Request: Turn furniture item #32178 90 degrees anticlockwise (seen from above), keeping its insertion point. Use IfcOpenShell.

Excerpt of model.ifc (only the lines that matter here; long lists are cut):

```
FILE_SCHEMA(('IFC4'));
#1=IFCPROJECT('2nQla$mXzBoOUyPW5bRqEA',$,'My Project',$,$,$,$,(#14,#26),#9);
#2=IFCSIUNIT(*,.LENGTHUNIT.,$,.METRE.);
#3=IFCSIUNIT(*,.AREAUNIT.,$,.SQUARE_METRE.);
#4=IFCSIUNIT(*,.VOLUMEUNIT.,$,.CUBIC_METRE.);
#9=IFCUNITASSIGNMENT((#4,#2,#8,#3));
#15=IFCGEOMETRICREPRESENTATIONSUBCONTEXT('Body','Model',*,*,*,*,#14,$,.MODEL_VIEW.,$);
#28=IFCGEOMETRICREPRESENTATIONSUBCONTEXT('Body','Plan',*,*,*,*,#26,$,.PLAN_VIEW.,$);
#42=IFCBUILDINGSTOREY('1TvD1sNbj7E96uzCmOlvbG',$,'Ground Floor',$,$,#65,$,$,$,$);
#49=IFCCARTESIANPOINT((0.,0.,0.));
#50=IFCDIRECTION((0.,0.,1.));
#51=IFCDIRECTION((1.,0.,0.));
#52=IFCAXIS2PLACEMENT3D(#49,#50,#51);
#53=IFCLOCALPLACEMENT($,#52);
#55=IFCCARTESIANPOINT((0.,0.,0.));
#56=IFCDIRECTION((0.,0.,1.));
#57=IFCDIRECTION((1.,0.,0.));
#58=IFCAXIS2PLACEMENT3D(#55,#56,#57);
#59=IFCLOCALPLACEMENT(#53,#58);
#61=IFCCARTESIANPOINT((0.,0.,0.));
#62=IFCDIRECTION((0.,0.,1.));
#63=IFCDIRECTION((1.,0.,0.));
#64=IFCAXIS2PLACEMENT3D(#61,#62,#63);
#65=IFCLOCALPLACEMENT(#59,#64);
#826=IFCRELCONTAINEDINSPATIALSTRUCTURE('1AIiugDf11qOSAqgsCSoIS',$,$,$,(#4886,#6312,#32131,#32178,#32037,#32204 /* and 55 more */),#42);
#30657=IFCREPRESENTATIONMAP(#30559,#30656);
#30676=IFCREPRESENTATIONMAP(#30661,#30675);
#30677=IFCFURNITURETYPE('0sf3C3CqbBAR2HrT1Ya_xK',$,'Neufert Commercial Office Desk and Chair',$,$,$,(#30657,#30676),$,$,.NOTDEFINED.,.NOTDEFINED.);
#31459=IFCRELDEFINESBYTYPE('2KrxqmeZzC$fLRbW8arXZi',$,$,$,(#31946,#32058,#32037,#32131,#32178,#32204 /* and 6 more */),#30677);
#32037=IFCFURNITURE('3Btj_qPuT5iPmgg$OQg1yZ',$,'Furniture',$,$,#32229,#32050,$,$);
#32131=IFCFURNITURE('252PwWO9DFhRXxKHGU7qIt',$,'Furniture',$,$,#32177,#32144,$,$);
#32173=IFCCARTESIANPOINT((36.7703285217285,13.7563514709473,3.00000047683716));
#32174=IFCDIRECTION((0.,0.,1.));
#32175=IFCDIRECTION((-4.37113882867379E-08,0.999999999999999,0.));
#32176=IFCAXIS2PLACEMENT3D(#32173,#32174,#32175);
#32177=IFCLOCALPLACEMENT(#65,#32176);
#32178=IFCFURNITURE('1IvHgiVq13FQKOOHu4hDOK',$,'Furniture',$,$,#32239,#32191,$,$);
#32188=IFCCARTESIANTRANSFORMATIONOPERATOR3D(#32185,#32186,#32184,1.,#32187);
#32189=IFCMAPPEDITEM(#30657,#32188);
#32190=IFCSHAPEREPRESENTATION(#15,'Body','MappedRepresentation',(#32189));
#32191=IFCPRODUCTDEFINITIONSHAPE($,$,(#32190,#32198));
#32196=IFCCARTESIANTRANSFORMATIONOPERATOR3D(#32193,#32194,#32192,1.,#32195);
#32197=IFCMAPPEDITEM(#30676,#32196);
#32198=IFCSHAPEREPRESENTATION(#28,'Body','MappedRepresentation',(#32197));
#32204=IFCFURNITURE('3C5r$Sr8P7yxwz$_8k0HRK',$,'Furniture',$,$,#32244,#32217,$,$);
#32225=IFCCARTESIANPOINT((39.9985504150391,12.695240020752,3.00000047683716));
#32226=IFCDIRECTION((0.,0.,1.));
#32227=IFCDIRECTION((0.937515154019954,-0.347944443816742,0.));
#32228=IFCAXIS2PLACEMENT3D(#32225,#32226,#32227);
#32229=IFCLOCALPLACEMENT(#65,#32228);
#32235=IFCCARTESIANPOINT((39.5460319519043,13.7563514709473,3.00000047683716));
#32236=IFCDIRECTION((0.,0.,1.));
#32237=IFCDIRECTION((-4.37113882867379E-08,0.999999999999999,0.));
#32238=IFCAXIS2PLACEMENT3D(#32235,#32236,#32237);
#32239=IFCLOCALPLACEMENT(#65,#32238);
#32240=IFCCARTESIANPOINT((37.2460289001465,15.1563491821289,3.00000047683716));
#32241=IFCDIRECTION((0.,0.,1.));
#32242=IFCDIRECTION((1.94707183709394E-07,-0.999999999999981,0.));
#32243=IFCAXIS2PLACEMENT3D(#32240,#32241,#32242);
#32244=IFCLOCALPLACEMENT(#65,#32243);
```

```python
import ifcopenshell
import ifcopenshell.api.geometry
import ifcopenshell.util.placement

model = ifcopenshell.open("model.ifc")

item = model.by_id(32178)
matrix = ifcopenshell.util.placement.get_local_placement(item.ObjectPlacement)
matrix = matrix @ ifcopenshell.util.placement.rotation(90, "Z")
ifcopenshell.api.geometry.edit_object_placement(model, product=item, matrix=matrix, is_si=False)

print(ifcopenshell.util.placement.get_local_placement(item.ObjectPlacement).round(3) + 0.0)

model.write("model_updated.ifc")
```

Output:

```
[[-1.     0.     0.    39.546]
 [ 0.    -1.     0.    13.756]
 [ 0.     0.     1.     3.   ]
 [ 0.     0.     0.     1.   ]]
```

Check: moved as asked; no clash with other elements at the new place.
